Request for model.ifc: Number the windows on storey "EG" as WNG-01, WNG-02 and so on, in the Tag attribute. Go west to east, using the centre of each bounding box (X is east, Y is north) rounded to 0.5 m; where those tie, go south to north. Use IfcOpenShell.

First a look at what the model holds.

```python
import ifcopenshell
import ifcopenshell.util.element
import ifcopenshell.util.placement

model = ifcopenshell.open("model.ifc")
print(model.schema)
storey = next(s for s in model.by_type("IfcBuildingStorey") if s.Name == "EG")
windows = [e for e in ifcopenshell.util.element.get_decomposition(storey) if e.is_a("IfcWindow")]
for e in sorted(windows, key=lambda e: e.id()):
    origin = ifcopenshell.util.placement.get_local_placement(e.ObjectPlacement)[:3, 3]
    print(e.id(), e.Tag, e.Name, origin.round(2) + 0.0, sep=" | ")
```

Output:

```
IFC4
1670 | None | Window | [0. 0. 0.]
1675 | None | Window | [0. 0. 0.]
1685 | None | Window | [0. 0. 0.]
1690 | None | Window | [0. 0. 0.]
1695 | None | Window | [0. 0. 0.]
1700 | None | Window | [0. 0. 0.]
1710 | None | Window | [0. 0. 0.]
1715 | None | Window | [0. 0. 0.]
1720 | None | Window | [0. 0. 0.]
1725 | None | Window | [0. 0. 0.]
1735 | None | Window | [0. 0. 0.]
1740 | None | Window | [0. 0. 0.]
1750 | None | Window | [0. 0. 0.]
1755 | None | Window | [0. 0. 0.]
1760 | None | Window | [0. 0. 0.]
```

```python
import ifcopenshell
import ifcopenshell.geom
import ifcopenshell.util.element
import ifcopenshell.util.shape

model = ifcopenshell.open("model.ifc")
settings = ifcopenshell.geom.settings()
settings.set("use-world-coords", True)


def centre(element):
    shape = ifcopenshell.geom.create_shape(settings, element)
    return ifcopenshell.util.shape.get_bbox_centroid(shape.geometry)


storey = next(s for s in model.by_type("IfcBuildingStorey") if s.Name == "EG")
windows = [e for e in ifcopenshell.util.element.get_decomposition(storey) if e.is_a("IfcWindow")]

# Insertion points can sit at a corner or the storey origin, so sort by the geometry (in metres).
centres = {e: centre(e) for e in windows}
windows.sort(key=lambda e: (round(centres[e][0] / 0.5), centres[e][1]))

for i, e in enumerate(windows, start=1):
    number = f"WNG-{i:02d}"
    e.Tag = number
    print(e.id(), number)

model.write("model_edited.ifc")
```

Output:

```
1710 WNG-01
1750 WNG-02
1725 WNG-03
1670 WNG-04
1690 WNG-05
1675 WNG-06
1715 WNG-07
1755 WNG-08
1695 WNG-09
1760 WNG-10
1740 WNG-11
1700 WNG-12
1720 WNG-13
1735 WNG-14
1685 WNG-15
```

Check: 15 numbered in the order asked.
